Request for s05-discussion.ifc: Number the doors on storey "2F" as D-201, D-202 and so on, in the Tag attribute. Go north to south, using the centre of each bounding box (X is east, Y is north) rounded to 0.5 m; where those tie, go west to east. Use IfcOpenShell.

First a look at what the model holds.

```python
import ifcopenshell
import ifcopenshell.util.element
import ifcopenshell.util.placement

model = ifcopenshell.open("s05-discussion.ifc")
print(model.schema)
storey = next(s for s in model.by_type("IfcBuildingStorey") if s.Name == "2F")
doors = [e for e in ifcopenshell.util.element.get_decomposition(storey) if e.is_a("IfcDoor")]
for e in sorted(doors, key=lambda e: e.id()):
    origin = ifcopenshell.util.placement.get_local_placement(e.ObjectPlacement)[:3, 3]
    print(e.id(), e.Tag, e.Name, origin.round(2) + 0.0, sep=" | ")
```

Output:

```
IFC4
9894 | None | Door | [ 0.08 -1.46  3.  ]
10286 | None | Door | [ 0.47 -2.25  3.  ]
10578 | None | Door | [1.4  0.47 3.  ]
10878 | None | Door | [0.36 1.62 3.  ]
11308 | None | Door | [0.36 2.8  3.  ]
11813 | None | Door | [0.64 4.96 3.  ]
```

```python
import ifcopenshell
import ifcopenshell.geom
import ifcopenshell.util.element
import ifcopenshell.util.shape

model = ifcopenshell.open("s05-discussion.ifc")
settings = ifcopenshell.geom.settings()
settings.set("use-world-coords", True)


def centre(element):
    shape = ifcopenshell.geom.create_shape(settings, element)
    return ifcopenshell.util.shape.get_bbox_centroid(shape.geometry)


storey = next(s for s in model.by_type("IfcBuildingStorey") if s.Name == "2F")
doors = [e for e in ifcopenshell.util.element.get_decomposition(storey) if e.is_a("IfcDoor")]

# Insertion points can sit at a corner or the storey origin, so sort by the geometry (in metres).
centres = {e: centre(e) for e in doors}
doors.sort(key=lambda e: (-round(centres[e][1] / 0.5), centres[e][0]))

for i, e in enumerate(doors, start=1):
    number = f"D-2{i:02d}"
    e.Tag = number
    print(e.id(), number)

model.write("s05-discussion_updated.ifc")
```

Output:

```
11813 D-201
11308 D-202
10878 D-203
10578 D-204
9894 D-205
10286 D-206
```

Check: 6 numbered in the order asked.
